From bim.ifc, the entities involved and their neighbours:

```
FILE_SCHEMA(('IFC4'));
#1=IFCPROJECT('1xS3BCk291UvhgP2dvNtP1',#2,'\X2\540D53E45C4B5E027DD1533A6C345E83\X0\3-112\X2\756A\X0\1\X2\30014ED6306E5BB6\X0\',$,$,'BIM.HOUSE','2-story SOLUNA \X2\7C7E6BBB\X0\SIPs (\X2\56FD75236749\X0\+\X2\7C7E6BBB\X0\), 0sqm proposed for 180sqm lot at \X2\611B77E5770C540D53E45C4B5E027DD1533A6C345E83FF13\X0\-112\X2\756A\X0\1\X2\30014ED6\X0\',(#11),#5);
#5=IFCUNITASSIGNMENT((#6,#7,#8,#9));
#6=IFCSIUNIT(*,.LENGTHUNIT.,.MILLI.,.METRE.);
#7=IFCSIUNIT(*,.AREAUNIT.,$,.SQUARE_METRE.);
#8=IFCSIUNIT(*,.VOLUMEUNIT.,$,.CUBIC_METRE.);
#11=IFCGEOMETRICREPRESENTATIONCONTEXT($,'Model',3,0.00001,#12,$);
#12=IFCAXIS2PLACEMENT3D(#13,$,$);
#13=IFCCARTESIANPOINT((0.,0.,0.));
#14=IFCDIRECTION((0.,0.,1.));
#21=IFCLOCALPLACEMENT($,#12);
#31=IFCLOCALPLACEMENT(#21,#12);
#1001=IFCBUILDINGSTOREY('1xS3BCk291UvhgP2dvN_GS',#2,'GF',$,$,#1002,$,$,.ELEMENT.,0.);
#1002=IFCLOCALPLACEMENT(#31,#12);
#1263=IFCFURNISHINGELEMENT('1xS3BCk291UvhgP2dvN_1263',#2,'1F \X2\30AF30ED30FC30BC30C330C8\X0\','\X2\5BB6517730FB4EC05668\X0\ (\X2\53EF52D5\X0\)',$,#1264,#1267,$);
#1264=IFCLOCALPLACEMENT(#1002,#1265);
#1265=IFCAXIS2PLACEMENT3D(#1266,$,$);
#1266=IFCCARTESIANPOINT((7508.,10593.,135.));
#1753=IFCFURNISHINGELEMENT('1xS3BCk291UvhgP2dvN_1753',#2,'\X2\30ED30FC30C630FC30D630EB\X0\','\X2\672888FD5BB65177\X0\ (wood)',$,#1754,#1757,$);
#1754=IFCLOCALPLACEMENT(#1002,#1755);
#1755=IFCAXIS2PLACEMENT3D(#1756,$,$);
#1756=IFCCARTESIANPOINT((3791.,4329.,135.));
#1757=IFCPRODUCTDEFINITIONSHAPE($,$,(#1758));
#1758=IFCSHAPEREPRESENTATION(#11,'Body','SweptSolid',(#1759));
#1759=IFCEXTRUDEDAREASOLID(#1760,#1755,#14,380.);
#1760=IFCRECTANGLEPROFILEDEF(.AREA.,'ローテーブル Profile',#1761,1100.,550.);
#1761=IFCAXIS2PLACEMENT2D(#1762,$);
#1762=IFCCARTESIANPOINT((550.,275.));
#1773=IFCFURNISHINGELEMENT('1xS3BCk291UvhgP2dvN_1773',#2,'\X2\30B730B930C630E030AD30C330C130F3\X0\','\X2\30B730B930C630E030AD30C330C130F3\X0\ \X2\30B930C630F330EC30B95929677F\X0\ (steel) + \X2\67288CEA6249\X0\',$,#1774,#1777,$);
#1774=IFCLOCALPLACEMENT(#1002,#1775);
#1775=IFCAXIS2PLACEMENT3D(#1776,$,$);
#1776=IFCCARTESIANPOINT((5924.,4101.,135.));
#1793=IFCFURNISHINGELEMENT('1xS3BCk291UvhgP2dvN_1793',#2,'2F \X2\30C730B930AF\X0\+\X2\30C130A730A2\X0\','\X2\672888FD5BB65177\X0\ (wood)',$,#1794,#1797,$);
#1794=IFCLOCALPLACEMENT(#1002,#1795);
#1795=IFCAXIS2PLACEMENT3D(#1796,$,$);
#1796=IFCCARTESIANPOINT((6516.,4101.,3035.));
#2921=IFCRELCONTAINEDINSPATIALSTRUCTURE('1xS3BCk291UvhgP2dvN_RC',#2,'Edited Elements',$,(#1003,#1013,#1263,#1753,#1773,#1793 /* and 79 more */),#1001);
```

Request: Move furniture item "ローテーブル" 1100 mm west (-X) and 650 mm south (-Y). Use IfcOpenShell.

```python
import ifcopenshell
import ifcopenshell.api.geometry
import ifcopenshell.util.placement

model = ifcopenshell.open("bim.ifc")

item = model.by_id(1753)
matrix = ifcopenshell.util.placement.get_local_placement(item.ObjectPlacement)
matrix[0, 3] -= 1100.0
matrix[1, 3] -= 650.0
ifcopenshell.api.geometry.edit_object_placement(model, product=item, matrix=matrix, is_si=False)

print(ifcopenshell.util.placement.get_local_placement(item.ObjectPlacement).round(3) + 0.0)

model.write("bim_rev.ifc")
```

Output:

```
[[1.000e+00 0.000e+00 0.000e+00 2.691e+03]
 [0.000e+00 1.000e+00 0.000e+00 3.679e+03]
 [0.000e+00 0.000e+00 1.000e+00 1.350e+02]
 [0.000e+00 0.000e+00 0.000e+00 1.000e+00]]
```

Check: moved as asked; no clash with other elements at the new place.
